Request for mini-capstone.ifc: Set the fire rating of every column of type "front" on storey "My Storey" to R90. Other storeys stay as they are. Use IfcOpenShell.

First a look at what the model holds.

```python
import ifcopenshell
import ifcopenshell.util.element

model = ifcopenshell.open("mini-capstone.ifc")
print(model.schema)
storey = next(s for s in model.by_type("IfcBuildingStorey") if s.Name == "My Storey")
columns = [e for e in ifcopenshell.util.element.get_decomposition(storey) if e.is_a("IfcColumn")]
seen = {}
for e in columns:
    element_type = ifcopenshell.util.element.get_type(e)
    key = (element_type.Name if element_type != e and element_type else None, ifcopenshell.util.element.get_pset(e, "Pset_ColumnCommon", "FireRating"))
    seen[key] = seen.get(key, 0) + 1
for (name, value), count in sorted(seen.items(), key=str):
    print(count, "x", name, "|", value)
```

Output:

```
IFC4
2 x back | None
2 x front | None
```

```python
import ifcopenshell
import ifcopenshell.api.pset
import ifcopenshell.util.element

model = ifcopenshell.open("mini-capstone.ifc")

storey = next(s for s in model.by_type("IfcBuildingStorey") if s.Name == "My Storey")
columns = [e for e in ifcopenshell.util.element.get_decomposition(storey) if e.is_a("IfcColumn")]

count = 0
for e in columns:
    element_type = ifcopenshell.util.element.get_type(e)
    if element_type in (None, e) or element_type.Name != "front":
        continue
    # add_pset returns the element's existing set when there is one.
    pset = ifcopenshell.api.pset.add_pset(model, product=e, name="Pset_ColumnCommon")
    ifcopenshell.api.pset.edit_pset(model, pset=pset, properties={"FireRating": "R90"})
    count += 1

print(count, "columns updated")

model.write("mini-capstone_edited.ifc")
```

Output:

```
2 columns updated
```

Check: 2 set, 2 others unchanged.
